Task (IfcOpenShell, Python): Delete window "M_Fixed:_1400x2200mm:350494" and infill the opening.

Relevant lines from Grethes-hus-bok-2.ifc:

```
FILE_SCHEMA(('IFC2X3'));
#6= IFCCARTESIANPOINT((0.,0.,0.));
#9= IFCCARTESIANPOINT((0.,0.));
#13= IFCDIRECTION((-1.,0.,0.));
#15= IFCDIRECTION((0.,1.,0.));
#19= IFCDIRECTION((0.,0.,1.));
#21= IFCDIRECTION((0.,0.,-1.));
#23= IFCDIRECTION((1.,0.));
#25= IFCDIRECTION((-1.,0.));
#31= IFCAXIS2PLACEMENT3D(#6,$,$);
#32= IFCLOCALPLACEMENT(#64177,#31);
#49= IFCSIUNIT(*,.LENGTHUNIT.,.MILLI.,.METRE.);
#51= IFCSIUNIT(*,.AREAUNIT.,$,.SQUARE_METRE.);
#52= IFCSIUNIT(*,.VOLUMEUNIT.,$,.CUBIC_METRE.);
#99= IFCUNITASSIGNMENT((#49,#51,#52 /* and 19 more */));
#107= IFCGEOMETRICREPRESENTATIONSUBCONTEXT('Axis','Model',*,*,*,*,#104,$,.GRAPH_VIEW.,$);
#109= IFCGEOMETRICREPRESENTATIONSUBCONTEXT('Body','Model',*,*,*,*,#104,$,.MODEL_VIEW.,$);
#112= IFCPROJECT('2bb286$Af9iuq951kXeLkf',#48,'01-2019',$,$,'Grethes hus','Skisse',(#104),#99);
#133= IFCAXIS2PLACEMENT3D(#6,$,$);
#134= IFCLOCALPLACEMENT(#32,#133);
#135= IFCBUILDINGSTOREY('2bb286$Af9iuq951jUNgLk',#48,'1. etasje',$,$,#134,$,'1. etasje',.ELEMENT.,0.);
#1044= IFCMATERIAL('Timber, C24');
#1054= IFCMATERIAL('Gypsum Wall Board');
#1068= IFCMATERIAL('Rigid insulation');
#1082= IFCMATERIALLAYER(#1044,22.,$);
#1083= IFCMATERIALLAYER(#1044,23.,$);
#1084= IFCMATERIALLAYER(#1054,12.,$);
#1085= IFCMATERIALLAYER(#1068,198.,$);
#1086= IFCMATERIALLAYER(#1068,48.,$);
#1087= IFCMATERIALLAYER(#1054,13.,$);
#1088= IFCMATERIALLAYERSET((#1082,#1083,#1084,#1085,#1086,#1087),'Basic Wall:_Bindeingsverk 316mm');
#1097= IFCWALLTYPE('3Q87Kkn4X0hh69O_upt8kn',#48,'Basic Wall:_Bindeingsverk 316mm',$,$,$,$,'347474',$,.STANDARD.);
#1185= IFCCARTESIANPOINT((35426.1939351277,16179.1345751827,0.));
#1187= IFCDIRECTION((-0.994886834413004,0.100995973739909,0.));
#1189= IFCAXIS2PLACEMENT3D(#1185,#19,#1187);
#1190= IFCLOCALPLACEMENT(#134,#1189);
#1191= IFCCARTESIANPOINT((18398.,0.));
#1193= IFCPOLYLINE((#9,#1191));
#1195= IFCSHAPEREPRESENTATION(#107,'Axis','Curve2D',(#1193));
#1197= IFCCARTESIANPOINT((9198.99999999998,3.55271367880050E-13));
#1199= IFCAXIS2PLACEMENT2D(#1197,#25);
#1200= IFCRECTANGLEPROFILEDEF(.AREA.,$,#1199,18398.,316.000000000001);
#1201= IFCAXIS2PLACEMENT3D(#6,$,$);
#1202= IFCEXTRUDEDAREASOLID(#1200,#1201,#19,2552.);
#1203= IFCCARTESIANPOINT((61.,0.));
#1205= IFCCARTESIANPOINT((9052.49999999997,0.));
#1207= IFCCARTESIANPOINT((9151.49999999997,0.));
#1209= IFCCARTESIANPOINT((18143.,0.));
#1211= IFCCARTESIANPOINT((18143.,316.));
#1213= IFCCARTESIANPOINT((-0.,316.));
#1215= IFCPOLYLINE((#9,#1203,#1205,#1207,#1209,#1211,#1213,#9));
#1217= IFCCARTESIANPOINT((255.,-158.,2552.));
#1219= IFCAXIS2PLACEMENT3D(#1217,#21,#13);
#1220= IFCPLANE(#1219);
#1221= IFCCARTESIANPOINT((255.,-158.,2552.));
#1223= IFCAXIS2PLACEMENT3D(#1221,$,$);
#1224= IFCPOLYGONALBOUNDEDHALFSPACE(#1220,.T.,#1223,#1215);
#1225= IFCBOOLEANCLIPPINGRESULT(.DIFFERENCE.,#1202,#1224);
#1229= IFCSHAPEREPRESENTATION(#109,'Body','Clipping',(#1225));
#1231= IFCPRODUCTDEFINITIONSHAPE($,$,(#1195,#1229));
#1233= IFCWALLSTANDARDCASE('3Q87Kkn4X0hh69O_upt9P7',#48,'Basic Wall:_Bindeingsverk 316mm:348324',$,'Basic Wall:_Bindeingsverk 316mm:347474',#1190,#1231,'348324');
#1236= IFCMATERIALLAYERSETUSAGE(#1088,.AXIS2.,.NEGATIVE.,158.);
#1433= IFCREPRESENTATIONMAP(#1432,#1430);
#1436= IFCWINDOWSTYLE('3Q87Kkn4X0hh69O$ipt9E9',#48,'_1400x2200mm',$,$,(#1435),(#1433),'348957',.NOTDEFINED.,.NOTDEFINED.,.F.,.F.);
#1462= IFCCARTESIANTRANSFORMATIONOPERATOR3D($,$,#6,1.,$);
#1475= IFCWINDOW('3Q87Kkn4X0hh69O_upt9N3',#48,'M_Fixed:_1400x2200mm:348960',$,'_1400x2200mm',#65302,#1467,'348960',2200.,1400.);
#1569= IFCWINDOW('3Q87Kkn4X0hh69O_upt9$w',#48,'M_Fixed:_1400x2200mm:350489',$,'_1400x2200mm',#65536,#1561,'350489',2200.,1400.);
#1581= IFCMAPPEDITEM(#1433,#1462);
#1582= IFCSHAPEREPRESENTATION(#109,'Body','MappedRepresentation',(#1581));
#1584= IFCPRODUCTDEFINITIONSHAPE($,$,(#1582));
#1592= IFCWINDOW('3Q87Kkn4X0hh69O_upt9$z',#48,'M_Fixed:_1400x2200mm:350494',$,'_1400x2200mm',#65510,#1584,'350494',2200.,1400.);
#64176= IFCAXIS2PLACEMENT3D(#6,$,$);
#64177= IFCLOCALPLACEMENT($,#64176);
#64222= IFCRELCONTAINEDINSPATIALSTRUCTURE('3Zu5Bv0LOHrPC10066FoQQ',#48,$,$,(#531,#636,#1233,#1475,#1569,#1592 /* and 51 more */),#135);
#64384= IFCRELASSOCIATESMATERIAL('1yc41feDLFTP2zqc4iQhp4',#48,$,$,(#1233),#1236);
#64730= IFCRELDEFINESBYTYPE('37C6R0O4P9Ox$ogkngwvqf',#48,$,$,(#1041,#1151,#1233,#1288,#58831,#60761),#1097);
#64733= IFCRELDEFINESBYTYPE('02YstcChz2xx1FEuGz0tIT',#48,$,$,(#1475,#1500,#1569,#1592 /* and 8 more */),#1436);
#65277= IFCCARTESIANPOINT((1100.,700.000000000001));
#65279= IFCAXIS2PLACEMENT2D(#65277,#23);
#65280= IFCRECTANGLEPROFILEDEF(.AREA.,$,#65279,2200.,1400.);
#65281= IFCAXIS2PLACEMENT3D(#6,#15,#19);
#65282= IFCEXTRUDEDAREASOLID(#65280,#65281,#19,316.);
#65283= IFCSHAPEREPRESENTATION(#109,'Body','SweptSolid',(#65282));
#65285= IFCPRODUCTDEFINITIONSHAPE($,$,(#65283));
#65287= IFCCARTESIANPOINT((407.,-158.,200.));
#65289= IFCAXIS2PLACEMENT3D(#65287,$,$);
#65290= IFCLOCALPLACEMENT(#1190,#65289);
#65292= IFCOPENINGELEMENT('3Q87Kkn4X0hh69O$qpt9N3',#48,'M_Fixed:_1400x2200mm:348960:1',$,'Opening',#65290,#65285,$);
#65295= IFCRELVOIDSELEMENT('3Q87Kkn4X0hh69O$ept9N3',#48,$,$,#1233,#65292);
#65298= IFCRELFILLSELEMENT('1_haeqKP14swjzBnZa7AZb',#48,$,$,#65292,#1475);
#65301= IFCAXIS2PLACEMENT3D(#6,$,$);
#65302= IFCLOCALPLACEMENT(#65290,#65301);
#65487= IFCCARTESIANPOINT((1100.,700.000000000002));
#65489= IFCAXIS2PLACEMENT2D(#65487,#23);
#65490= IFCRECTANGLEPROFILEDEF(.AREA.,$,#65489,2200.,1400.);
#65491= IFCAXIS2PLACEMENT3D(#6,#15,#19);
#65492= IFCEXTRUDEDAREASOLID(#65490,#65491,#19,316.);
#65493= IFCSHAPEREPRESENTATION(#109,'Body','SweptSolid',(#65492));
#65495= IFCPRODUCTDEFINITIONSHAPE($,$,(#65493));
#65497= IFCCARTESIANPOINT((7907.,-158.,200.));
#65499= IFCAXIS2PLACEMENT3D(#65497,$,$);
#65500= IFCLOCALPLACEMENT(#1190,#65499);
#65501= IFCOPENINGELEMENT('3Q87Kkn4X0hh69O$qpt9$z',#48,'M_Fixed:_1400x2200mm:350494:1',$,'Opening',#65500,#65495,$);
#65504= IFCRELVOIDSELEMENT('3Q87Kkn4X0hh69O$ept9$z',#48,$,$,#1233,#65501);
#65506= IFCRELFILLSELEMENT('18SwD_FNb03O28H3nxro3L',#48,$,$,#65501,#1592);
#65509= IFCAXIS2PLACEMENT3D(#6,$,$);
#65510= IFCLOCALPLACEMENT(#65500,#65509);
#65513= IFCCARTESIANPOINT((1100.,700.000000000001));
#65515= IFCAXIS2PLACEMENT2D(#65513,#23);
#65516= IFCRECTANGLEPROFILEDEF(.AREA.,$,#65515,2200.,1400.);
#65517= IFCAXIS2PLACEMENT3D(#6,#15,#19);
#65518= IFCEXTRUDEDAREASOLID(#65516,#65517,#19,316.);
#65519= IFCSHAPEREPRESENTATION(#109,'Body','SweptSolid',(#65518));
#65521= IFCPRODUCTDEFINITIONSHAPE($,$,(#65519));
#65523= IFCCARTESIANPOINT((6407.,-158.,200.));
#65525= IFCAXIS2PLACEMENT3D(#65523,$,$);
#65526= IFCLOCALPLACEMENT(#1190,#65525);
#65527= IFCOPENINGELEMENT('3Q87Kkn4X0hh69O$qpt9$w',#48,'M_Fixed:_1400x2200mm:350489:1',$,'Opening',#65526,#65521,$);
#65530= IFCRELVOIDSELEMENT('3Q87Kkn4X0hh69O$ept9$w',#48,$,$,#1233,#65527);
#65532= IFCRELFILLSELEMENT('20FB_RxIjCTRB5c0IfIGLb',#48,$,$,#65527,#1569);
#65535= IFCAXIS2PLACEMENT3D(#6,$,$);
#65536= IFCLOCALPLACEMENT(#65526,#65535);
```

```python
import ifcopenshell
import ifcopenshell.api.feature
import ifcopenshell.api.root
import ifcopenshell.geom
import ifcopenshell.util.shape

model = ifcopenshell.open("Grethes-hus-bok-2.ifc")
settings = ifcopenshell.geom.settings()


def volume(element):
    """Net volume in cubic metres, openings subtracted."""
    shape = ifcopenshell.geom.create_shape(settings, element)
    return ifcopenshell.util.shape.get_volume(shape.geometry)


window = model.by_guid("3Q87Kkn4X0hh69O_upt9$z")
opening = window.FillsVoids[0].RelatingOpeningElement
wall = opening.VoidsElements[0].RelatingBuildingElement
before = volume(wall)

ifcopenshell.api.root.remove_product(model, product=window)
ifcopenshell.api.feature.remove_feature(model, feature=opening)

after = volume(wall)

print(f"wall volume {before:.3f} -> {after:.3f} m3")

model.write("Grethes-hus-bok-2_updated.ifc")
```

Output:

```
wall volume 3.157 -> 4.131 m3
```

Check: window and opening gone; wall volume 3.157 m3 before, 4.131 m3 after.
